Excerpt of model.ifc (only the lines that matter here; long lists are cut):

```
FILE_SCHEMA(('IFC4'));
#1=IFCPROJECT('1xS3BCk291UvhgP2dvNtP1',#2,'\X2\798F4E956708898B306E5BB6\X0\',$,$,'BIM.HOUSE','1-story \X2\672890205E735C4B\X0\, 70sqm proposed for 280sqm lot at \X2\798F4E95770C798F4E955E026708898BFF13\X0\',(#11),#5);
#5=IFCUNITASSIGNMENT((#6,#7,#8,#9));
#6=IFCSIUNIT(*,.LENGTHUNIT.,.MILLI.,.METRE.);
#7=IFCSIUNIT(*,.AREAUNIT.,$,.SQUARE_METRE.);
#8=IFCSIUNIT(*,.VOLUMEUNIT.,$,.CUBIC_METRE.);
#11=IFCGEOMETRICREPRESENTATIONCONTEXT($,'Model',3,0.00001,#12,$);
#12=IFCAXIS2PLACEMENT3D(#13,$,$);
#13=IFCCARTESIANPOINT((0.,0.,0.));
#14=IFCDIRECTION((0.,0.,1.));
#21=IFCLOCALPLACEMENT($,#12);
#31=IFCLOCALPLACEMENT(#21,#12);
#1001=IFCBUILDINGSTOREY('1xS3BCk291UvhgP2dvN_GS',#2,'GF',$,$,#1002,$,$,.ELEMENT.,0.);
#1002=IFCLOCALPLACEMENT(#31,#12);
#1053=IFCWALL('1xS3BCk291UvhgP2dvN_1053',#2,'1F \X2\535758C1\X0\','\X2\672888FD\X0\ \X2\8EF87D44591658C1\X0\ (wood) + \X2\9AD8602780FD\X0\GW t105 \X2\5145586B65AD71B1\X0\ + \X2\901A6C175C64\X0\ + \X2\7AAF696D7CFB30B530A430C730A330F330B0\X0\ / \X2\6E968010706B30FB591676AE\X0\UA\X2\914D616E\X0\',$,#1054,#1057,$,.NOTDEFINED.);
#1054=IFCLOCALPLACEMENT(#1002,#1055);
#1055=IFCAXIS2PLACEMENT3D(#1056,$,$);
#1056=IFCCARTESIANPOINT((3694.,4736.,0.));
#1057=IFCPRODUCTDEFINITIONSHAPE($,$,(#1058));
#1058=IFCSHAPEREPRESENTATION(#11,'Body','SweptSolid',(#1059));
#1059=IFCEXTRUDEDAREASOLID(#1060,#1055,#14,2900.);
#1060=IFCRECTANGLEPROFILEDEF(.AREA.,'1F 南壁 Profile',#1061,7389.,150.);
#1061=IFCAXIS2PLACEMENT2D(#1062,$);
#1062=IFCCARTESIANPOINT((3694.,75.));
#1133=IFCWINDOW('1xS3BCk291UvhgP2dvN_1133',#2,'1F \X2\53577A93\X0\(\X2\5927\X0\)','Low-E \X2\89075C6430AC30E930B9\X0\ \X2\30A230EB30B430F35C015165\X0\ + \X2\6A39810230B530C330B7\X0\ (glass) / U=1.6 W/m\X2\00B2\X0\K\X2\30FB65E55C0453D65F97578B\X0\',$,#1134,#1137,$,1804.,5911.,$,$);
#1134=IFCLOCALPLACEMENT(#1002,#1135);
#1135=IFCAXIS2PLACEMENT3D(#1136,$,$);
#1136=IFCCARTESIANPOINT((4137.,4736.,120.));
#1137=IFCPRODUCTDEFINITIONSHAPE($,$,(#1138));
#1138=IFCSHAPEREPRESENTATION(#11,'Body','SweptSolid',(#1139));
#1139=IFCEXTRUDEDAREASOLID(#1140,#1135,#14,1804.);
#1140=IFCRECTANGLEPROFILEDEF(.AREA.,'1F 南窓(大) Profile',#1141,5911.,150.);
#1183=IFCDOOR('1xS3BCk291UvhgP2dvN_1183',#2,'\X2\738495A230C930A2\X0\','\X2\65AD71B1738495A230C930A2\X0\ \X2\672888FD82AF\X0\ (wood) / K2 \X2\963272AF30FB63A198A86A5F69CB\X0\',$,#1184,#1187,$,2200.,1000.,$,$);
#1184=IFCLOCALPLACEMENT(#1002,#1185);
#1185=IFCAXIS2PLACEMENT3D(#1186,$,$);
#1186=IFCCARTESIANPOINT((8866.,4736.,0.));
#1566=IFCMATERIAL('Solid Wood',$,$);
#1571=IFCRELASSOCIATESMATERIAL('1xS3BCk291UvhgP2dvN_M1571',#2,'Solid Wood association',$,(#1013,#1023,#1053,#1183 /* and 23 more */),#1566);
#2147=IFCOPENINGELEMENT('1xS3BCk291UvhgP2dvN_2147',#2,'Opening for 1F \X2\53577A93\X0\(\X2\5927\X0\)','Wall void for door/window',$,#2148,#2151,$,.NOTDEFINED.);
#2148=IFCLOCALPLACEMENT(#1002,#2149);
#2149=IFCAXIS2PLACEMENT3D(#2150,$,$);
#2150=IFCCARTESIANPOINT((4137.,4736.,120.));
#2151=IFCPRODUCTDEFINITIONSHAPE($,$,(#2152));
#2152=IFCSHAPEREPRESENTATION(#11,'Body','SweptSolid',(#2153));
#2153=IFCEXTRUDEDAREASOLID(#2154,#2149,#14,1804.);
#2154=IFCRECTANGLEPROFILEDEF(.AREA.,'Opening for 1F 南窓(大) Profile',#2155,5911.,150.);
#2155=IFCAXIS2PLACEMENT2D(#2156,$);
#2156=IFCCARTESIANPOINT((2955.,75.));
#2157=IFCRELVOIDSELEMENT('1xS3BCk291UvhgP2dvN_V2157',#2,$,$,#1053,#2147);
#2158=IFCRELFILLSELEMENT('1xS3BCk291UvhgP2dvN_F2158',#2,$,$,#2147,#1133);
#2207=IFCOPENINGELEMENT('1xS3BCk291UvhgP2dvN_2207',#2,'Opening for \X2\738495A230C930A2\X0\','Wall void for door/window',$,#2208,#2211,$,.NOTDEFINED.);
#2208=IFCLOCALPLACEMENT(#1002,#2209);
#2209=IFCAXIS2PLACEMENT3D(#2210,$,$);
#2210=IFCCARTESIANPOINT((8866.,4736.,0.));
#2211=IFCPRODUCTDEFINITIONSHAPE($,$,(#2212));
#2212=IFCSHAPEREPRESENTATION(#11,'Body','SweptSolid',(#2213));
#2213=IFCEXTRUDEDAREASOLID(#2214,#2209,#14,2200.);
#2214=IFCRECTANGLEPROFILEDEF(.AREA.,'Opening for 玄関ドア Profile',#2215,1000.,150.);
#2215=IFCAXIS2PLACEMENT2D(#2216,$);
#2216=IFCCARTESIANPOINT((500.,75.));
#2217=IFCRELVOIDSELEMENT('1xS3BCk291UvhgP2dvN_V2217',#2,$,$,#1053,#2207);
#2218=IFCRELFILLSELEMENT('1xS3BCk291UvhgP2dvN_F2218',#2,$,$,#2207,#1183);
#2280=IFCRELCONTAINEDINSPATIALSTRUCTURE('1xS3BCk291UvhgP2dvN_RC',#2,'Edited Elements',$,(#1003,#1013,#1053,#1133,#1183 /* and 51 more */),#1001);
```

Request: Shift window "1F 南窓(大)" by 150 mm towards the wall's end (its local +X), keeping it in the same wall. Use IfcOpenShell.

```python
import ifcopenshell
import ifcopenshell.api.geometry
import ifcopenshell.util.placement
import ifcopenshell.util.unit

model = ifcopenshell.open("model.ifc")
unit_scale = ifcopenshell.util.unit.calculate_unit_scale(model)

window = model.by_guid("1xS3BCk291UvhgP2dvN_1133")
opening = window.FillsVoids[0].RelatingOpeningElement
wall = opening.VoidsElements[0].RelatingBuildingElement

wall_matrix = ifcopenshell.util.placement.get_local_placement(wall.ObjectPlacement)
shift = wall_matrix[:3, 0] * 0.15 / unit_scale
before = ifcopenshell.util.placement.get_local_placement(window.ObjectPlacement)[:3, 3].copy()

# The window is not placed relative to its opening, so move both.
for product in (opening, window):
    matrix = ifcopenshell.util.placement.get_local_placement(product.ObjectPlacement)
    matrix[:3, 3] += shift
    ifcopenshell.api.geometry.edit_object_placement(model, product=product, matrix=matrix, is_si=False)

after = ifcopenshell.util.placement.get_local_placement(window.ObjectPlacement)[:3, 3]
print("window moved by", (after - before).round(3) + 0.0)

model.write("model_rev.ifc")
```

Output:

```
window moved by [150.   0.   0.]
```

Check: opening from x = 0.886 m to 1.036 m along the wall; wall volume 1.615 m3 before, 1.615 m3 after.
